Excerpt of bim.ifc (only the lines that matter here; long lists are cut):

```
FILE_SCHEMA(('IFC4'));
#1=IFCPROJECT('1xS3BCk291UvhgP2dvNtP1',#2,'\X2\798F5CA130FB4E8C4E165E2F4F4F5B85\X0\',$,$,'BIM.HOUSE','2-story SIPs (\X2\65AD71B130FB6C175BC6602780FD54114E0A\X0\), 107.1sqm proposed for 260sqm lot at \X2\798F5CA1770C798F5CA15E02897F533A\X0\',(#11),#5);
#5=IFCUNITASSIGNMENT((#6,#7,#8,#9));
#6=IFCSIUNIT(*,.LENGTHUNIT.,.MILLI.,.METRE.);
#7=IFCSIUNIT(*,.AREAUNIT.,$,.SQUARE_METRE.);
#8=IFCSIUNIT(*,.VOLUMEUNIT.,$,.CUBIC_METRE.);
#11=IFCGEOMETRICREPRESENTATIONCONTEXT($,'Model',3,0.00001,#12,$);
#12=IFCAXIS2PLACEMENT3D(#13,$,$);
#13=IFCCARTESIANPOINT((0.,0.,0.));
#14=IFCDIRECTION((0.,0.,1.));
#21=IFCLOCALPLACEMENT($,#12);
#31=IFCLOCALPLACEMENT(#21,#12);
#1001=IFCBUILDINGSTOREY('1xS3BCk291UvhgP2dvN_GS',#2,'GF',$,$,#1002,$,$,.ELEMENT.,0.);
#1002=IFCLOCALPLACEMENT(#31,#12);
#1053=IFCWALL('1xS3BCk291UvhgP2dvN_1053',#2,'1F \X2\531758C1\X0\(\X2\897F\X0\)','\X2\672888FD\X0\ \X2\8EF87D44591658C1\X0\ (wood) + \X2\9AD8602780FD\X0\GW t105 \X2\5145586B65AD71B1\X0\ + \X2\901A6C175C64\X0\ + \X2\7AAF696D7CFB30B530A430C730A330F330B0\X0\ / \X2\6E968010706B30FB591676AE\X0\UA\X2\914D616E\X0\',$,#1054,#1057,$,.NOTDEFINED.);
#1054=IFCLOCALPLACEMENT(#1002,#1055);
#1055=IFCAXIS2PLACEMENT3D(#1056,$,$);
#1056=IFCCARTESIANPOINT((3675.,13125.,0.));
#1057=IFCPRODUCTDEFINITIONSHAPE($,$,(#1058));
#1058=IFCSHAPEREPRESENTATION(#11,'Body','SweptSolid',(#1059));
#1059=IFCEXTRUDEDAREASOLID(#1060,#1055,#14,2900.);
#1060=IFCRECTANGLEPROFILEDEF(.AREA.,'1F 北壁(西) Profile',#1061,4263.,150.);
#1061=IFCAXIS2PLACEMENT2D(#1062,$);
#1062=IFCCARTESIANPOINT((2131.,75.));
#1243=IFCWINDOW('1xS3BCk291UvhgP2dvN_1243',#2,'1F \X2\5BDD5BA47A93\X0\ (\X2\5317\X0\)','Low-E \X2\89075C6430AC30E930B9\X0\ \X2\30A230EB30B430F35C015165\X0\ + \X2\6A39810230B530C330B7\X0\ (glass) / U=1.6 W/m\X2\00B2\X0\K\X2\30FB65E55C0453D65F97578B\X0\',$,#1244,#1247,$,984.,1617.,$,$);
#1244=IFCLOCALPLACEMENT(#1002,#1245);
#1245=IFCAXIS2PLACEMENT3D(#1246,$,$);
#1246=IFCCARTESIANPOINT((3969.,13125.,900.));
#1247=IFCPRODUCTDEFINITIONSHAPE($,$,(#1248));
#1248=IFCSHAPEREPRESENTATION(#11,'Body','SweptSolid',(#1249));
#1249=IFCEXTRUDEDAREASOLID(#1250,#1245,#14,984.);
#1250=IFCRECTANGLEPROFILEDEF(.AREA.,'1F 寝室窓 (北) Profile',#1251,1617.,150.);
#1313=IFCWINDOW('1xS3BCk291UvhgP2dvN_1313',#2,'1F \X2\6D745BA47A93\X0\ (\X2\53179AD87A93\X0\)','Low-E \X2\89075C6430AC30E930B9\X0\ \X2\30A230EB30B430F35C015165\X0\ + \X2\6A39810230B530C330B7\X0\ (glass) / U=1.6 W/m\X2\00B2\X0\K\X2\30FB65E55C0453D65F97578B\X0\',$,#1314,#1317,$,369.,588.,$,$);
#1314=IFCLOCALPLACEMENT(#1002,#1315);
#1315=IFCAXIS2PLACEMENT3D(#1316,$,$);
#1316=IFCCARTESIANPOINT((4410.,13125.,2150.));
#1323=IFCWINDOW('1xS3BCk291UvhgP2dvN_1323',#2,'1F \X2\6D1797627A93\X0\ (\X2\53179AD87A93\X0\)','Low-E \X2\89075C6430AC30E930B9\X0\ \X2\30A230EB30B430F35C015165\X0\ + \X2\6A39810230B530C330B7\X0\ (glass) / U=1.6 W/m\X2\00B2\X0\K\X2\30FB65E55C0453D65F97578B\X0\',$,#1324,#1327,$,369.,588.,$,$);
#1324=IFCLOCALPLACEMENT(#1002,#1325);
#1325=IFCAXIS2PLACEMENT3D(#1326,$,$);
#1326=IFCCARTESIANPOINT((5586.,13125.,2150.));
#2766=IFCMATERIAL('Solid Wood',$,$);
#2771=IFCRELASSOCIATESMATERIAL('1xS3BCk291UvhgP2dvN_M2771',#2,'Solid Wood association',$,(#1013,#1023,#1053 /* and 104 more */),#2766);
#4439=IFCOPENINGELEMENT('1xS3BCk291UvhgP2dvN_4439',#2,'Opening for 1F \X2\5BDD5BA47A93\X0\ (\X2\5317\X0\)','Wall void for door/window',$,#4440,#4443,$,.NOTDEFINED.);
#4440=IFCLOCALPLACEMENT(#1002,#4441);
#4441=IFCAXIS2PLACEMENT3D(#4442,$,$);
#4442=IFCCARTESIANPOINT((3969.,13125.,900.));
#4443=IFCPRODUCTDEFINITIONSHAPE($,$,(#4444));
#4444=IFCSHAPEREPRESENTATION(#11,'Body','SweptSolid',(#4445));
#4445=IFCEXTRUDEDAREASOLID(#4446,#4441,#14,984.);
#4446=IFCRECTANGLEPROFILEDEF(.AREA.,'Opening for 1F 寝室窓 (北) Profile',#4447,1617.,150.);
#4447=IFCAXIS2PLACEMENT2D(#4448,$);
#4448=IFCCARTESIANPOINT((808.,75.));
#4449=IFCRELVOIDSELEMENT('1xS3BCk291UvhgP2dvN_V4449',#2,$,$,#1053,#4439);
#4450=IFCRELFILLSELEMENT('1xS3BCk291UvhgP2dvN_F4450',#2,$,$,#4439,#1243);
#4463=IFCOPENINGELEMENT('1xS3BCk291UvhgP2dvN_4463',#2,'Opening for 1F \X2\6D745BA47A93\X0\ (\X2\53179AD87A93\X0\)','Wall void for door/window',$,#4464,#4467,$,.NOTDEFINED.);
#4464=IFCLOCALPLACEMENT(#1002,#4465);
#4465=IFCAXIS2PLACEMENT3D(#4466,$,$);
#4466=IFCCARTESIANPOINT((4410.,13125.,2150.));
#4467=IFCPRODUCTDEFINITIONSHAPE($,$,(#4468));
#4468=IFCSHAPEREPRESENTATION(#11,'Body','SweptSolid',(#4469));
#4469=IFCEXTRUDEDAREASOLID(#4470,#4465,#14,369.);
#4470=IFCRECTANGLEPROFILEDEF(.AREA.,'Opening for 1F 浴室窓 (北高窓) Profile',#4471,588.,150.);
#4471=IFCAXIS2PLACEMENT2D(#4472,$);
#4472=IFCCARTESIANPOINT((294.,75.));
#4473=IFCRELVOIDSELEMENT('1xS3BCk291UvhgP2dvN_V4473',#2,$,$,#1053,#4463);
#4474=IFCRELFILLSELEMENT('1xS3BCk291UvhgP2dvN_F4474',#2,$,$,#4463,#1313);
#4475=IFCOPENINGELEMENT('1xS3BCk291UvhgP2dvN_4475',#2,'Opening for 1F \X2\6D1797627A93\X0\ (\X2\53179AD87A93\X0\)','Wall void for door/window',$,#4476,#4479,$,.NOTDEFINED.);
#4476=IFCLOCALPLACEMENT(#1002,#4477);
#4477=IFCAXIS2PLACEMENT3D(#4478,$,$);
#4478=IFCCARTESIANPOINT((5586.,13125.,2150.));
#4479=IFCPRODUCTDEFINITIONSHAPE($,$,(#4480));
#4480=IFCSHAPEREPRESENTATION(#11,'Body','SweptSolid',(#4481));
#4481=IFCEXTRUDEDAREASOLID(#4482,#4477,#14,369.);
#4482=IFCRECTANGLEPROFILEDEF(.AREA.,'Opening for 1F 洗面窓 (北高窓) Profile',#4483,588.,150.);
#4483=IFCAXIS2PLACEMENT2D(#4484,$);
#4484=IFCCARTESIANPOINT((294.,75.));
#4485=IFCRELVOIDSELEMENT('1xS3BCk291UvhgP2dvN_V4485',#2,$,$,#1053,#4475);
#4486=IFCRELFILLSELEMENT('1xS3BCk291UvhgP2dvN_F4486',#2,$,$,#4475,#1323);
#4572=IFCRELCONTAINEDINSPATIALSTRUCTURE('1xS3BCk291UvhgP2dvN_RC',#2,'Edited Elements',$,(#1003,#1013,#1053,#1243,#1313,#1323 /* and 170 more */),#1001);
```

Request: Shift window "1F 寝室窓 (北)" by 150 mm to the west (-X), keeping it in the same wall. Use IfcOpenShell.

```python
import ifcopenshell
import ifcopenshell.api.geometry
import ifcopenshell.util.placement

model = ifcopenshell.open("bim.ifc")

window = model.by_guid("1xS3BCk291UvhgP2dvN_1243")
opening = window.FillsVoids[0].RelatingOpeningElement
wall = opening.VoidsElements[0].RelatingBuildingElement

wall_matrix = ifcopenshell.util.placement.get_local_placement(wall.ObjectPlacement)
shift = wall_matrix[:3, 0] * -150.0
before = ifcopenshell.util.placement.get_local_placement(window.ObjectPlacement)[:3, 3].copy()

# The window is not placed relative to its opening, so move both.
for product in (opening, window):
    matrix = ifcopenshell.util.placement.get_local_placement(product.ObjectPlacement)
    matrix[:3, 3] += shift
    ifcopenshell.api.geometry.edit_object_placement(model, product=product, matrix=matrix, is_si=False)

after = ifcopenshell.util.placement.get_local_placement(window.ObjectPlacement)[:3, 3]
print("window moved by", (after - before).round(3) + 0.0)

model.write("bim-out.ifc")
```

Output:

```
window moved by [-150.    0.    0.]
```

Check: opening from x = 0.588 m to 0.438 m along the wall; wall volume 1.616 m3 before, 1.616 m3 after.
